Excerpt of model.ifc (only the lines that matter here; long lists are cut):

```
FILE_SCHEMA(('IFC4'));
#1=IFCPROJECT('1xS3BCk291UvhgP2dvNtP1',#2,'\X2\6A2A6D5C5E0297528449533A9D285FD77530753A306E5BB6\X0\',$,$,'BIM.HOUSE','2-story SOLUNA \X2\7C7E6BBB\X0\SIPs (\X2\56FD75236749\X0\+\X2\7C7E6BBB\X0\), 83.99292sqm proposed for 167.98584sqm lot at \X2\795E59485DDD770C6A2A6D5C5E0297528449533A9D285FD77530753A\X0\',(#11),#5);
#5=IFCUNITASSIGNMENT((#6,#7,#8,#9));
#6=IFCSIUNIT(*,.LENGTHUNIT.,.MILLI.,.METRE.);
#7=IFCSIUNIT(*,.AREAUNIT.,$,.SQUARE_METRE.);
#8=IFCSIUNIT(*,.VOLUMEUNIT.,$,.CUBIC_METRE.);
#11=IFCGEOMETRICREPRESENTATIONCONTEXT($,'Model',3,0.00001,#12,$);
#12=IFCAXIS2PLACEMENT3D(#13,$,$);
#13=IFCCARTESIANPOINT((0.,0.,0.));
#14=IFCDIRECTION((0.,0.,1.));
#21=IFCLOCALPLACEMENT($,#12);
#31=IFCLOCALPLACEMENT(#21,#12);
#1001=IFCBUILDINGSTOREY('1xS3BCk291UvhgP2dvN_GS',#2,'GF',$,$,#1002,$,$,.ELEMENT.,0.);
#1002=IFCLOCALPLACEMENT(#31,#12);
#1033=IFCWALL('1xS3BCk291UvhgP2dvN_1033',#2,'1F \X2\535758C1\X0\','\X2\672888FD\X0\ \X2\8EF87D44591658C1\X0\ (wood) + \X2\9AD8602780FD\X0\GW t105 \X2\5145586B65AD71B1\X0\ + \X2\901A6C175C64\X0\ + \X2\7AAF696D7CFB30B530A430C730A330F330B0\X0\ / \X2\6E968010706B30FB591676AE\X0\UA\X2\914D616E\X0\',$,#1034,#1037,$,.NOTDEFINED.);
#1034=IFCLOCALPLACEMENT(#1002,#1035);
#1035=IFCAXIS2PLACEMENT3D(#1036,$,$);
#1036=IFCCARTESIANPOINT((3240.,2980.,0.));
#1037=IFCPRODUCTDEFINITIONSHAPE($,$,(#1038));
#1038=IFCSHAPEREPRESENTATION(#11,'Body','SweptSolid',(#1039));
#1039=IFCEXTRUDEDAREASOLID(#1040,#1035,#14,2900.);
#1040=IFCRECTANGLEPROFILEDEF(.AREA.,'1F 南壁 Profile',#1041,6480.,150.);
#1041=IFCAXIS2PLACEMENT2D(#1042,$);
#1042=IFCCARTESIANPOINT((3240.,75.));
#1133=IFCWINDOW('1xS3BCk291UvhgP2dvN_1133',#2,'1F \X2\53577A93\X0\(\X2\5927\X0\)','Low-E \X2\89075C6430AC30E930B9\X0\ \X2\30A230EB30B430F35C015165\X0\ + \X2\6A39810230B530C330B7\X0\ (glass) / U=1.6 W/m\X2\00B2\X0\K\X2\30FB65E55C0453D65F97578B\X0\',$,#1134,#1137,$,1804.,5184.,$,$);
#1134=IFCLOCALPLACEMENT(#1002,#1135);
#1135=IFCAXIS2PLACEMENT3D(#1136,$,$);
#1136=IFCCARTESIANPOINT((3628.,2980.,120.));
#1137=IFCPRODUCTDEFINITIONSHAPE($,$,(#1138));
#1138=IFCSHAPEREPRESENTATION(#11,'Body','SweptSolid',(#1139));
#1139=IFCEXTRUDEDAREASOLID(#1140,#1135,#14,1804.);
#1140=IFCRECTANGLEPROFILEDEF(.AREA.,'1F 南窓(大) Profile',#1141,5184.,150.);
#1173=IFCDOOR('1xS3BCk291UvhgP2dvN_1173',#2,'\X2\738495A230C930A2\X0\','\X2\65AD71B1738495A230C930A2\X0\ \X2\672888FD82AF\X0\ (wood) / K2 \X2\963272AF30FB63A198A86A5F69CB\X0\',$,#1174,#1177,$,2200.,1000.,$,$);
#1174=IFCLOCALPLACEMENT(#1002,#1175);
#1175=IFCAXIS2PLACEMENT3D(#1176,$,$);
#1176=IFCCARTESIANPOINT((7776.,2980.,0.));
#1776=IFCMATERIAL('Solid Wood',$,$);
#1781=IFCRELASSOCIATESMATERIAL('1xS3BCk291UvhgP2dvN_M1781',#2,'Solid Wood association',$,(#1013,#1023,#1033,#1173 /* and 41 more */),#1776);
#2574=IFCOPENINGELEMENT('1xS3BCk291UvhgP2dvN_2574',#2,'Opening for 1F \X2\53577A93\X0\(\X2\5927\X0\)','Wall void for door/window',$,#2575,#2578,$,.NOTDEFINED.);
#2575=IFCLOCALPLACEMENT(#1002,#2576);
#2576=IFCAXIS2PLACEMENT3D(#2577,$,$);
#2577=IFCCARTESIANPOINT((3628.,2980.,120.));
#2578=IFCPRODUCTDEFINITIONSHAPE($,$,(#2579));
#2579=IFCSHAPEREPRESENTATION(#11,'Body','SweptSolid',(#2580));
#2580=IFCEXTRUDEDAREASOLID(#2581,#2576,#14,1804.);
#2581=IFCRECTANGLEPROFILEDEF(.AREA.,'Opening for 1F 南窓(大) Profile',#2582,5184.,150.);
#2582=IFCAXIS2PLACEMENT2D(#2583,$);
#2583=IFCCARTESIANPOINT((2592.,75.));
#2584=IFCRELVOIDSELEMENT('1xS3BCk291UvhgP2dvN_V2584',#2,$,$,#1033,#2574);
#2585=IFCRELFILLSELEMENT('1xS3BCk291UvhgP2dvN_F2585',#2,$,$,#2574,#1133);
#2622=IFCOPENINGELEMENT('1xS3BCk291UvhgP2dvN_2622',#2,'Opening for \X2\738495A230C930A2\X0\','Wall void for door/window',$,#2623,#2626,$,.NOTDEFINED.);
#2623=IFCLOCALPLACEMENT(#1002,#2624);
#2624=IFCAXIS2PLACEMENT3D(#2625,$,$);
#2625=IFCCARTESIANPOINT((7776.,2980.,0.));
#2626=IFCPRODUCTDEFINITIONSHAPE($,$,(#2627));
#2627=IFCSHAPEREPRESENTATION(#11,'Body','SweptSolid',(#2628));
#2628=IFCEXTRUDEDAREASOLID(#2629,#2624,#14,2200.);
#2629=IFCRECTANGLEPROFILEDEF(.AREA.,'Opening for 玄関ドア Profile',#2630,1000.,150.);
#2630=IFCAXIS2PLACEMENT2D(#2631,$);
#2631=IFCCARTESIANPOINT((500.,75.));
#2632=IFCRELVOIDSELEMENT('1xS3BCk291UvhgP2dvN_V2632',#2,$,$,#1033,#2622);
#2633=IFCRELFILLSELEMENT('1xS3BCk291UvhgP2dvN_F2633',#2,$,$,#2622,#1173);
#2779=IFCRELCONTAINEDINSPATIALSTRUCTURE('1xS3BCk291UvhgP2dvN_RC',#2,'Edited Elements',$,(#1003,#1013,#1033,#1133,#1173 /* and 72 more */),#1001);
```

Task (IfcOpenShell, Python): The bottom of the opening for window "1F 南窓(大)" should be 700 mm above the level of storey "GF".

```python
import numpy as np
import ifcopenshell
import ifcopenshell.api.geometry
import ifcopenshell.geom
import ifcopenshell.util.element
import ifcopenshell.util.placement
import ifcopenshell.util.shape
import ifcopenshell.util.unit

model = ifcopenshell.open("model.ifc")
unit_scale = ifcopenshell.util.unit.calculate_unit_scale(model)

window = model.by_guid("1xS3BCk291UvhgP2dvN_1133")
opening = window.FillsVoids[0].RelatingOpeningElement
storey = ifcopenshell.util.element.get_container(window, ifc_class="IfcBuildingStorey")
level = ifcopenshell.util.placement.get_local_placement(storey.ObjectPlacement)[2, 3]

# The opening's origin need not be at the sill, so measure its lowest point.
shape = ifcopenshell.geom.create_shape(ifcopenshell.geom.settings(), opening)
bottom = ifcopenshell.util.shape.get_shape_bottom_elevation(shape, shape.geometry) / unit_scale
dz = level + 0.7 / unit_scale - bottom

shift = np.array([0.0, 0.0, dz])
# The window is not placed relative to its opening, so move both.
for product in (opening, window):
    matrix = ifcopenshell.util.placement.get_local_placement(product.ObjectPlacement)
    matrix[:3, 3] += shift
    ifcopenshell.api.geometry.edit_object_placement(model, product=product, matrix=matrix, is_si=False)

print(f"moved by {dz * unit_scale:+.3f} m")

model.write("model_updated.ifc")
```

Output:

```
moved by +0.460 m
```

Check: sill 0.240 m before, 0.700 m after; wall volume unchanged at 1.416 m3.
